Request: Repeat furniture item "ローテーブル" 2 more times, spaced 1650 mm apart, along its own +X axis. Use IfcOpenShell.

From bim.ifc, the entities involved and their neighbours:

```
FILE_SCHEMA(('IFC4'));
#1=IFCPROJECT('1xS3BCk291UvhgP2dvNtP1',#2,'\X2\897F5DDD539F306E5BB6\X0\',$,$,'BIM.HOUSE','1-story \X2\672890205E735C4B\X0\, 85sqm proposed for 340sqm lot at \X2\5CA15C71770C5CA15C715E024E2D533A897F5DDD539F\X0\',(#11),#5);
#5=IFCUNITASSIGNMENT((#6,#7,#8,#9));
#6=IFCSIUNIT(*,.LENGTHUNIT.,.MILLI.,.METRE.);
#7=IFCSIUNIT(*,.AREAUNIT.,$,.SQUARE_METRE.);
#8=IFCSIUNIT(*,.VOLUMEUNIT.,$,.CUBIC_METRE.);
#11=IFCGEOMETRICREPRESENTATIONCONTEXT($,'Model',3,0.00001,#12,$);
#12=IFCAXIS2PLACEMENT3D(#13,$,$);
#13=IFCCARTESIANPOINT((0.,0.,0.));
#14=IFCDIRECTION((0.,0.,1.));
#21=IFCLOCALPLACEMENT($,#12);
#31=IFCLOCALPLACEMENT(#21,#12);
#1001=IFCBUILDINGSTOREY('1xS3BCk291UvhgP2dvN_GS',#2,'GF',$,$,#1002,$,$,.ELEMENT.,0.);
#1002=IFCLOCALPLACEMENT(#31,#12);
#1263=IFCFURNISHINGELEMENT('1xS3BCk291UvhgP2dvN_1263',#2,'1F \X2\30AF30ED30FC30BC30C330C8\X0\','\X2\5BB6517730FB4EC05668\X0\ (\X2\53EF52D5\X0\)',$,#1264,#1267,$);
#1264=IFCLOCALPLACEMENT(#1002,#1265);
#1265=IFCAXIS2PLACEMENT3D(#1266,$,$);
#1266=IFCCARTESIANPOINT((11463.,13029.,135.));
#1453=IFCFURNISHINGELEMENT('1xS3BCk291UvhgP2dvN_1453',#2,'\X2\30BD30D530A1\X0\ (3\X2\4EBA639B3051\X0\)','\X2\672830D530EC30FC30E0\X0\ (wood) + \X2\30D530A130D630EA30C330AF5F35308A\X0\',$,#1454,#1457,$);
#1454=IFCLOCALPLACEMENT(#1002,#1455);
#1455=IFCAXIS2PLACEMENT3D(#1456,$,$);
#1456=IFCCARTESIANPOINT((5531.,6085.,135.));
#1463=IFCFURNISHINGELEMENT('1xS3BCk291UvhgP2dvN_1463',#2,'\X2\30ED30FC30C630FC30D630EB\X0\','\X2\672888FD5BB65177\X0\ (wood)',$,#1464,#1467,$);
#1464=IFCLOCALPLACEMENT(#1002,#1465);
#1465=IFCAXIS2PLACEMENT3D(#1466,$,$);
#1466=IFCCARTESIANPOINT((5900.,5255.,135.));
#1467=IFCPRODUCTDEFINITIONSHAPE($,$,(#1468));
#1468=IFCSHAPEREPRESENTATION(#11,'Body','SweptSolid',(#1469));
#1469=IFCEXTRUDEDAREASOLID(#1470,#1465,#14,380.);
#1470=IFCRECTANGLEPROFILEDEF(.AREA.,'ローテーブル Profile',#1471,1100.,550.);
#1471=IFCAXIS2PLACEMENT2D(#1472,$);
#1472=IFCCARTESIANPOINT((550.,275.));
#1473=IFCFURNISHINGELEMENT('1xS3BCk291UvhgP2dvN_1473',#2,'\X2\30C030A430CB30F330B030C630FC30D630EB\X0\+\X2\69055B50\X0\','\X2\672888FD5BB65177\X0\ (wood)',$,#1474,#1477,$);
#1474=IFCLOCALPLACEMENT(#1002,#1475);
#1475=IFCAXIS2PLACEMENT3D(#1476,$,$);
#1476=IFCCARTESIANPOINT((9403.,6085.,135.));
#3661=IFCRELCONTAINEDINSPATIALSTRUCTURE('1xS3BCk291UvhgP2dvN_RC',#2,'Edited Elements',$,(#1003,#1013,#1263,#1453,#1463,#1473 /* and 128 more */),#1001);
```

```python
import ifcopenshell
import ifcopenshell.api.geometry
import ifcopenshell.api.root
import ifcopenshell.util.element
import ifcopenshell.util.placement
import ifcopenshell.util.unit

model = ifcopenshell.open("bim.ifc")
unit_scale = ifcopenshell.util.unit.calculate_unit_scale(model)


def reuse_history(source, copy):
    """copy_class also copies each property set's owner history, people and application; keep the originals."""
    for rel in copy.IsDefinedBy:
        if rel.is_a("IfcRelDefinesByProperties") and (history := rel.RelatingPropertyDefinition.OwnerHistory):
            rel.RelatingPropertyDefinition.OwnerHistory = source.OwnerHistory
            ifcopenshell.util.element.remove_deep2(model, history)


source = model.by_guid("1xS3BCk291UvhgP2dvN_1463")
base = ifcopenshell.util.placement.get_local_placement(source.ObjectPlacement)
step = base[:3, 0] * 1.65 / unit_scale

for i in range(1, 3):
    copy = ifcopenshell.api.root.copy_class(model, product=source)
    copy.Representation = ifcopenshell.util.element.copy_deep(
        model, source.Representation, exclude=["IfcGeometricRepresentationContext", "IfcRepresentationMap"]
    )
    reuse_history(source, copy)
    matrix = base.copy()
    matrix[:3, 3] += i * step
    print("added at", matrix[:3, 3].round(3) + 0.0)
    ifcopenshell.api.geometry.edit_object_placement(model, product=copy, matrix=matrix, is_si=False)

model.write("bim-out.ifc")
```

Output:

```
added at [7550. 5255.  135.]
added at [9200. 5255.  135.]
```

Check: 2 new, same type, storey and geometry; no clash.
